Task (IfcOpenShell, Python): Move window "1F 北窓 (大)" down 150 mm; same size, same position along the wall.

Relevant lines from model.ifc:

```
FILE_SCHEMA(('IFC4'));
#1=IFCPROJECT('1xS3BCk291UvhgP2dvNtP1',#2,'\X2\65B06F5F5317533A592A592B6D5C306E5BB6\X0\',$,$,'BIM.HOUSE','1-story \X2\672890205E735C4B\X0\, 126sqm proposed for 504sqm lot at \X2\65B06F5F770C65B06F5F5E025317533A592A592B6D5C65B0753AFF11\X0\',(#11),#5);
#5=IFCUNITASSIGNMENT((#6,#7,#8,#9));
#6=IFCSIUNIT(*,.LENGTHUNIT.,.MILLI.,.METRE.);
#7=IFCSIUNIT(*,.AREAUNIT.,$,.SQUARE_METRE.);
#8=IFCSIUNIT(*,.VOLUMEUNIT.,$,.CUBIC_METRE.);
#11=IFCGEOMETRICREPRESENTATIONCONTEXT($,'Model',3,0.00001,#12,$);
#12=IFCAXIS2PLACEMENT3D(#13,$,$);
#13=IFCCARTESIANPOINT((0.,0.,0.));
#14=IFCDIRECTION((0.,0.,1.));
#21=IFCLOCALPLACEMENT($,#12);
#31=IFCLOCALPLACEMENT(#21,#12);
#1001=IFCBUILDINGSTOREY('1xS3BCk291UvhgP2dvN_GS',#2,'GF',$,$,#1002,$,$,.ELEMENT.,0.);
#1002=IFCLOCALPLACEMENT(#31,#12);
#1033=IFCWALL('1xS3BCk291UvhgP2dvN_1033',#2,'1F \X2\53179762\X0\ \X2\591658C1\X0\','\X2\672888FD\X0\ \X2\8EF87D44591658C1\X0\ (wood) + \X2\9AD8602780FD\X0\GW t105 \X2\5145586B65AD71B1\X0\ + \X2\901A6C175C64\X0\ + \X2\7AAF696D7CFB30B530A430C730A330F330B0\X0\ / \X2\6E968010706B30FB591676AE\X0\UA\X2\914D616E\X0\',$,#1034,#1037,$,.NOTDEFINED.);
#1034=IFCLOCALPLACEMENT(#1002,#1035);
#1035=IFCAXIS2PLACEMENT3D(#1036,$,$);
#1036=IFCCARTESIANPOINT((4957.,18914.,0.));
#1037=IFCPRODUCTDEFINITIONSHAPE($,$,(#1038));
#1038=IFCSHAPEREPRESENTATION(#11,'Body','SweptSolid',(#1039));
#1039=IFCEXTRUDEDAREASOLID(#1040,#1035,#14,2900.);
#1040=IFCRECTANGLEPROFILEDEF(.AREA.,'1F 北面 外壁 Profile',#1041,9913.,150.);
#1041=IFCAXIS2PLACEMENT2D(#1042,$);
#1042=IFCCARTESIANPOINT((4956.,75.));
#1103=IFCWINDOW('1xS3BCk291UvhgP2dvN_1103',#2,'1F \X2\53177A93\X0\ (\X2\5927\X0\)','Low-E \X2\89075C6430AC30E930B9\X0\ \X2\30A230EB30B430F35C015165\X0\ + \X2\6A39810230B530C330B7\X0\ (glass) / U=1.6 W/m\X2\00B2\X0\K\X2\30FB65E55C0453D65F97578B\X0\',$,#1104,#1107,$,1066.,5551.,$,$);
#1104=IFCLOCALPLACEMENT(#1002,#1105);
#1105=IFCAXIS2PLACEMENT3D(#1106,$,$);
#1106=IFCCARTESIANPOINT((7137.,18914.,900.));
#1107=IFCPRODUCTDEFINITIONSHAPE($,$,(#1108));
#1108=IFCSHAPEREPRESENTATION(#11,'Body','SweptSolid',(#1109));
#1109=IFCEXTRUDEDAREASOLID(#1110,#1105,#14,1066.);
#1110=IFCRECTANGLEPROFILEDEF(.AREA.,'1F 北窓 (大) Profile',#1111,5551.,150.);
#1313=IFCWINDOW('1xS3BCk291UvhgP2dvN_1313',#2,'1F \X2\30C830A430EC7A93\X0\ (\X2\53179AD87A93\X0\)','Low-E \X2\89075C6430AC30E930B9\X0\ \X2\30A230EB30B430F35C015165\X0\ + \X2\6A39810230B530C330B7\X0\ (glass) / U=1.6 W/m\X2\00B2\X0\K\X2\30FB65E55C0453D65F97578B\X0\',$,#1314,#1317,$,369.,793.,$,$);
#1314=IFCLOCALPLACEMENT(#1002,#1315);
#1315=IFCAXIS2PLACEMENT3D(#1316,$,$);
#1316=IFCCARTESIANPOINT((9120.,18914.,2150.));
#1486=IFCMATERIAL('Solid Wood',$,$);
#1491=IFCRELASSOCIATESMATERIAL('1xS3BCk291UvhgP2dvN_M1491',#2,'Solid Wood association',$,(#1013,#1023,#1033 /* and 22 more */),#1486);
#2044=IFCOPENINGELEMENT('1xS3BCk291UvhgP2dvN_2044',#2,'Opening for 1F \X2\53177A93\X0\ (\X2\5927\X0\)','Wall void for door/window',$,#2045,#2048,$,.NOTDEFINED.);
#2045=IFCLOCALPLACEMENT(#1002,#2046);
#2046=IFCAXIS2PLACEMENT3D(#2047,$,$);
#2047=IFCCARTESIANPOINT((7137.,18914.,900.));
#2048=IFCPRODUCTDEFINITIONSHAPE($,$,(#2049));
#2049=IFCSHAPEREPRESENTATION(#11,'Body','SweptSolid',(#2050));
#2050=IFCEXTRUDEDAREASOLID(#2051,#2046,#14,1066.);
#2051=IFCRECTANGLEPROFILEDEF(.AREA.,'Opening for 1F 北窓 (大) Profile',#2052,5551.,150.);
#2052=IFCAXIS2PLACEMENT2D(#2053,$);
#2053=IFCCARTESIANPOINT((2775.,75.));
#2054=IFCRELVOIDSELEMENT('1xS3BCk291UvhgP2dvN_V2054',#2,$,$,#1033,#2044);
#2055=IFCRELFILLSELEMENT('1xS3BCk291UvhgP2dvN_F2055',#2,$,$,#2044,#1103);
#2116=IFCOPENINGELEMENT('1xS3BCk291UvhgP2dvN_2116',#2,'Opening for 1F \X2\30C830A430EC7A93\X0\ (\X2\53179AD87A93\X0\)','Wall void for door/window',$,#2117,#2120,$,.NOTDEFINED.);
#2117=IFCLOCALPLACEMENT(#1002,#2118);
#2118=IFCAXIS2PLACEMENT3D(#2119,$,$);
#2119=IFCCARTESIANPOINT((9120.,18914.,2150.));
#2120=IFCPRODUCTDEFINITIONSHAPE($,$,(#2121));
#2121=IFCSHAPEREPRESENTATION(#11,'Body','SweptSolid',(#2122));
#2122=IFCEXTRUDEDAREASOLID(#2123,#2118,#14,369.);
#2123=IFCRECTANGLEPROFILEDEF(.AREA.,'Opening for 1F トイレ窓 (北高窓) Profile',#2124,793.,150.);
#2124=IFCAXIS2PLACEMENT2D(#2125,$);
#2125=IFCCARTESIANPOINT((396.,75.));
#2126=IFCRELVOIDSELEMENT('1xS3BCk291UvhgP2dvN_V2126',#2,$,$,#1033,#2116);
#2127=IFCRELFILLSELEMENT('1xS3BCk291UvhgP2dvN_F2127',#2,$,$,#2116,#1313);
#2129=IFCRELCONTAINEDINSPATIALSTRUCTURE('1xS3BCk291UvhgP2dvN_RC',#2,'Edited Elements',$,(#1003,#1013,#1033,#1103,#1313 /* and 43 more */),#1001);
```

```python
import numpy as np
import ifcopenshell
import ifcopenshell.api.geometry
import ifcopenshell.util.placement
import ifcopenshell.util.unit

model = ifcopenshell.open("model.ifc")
unit_scale = ifcopenshell.util.unit.calculate_unit_scale(model)

window = model.by_guid("1xS3BCk291UvhgP2dvN_1103")
opening = window.FillsVoids[0].RelatingOpeningElement
dz = -0.15 / unit_scale

shift = np.array([0.0, 0.0, dz])
# The window is not placed relative to its opening, so move both.
for product in (opening, window):
    matrix = ifcopenshell.util.placement.get_local_placement(product.ObjectPlacement)
    matrix[:3, 3] += shift
    ifcopenshell.api.geometry.edit_object_placement(model, product=product, matrix=matrix, is_si=False)

print(f"moved by {dz * unit_scale:+.3f} m")

model.write("model-out.ifc")
```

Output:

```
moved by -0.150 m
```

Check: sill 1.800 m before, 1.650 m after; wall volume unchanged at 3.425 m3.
